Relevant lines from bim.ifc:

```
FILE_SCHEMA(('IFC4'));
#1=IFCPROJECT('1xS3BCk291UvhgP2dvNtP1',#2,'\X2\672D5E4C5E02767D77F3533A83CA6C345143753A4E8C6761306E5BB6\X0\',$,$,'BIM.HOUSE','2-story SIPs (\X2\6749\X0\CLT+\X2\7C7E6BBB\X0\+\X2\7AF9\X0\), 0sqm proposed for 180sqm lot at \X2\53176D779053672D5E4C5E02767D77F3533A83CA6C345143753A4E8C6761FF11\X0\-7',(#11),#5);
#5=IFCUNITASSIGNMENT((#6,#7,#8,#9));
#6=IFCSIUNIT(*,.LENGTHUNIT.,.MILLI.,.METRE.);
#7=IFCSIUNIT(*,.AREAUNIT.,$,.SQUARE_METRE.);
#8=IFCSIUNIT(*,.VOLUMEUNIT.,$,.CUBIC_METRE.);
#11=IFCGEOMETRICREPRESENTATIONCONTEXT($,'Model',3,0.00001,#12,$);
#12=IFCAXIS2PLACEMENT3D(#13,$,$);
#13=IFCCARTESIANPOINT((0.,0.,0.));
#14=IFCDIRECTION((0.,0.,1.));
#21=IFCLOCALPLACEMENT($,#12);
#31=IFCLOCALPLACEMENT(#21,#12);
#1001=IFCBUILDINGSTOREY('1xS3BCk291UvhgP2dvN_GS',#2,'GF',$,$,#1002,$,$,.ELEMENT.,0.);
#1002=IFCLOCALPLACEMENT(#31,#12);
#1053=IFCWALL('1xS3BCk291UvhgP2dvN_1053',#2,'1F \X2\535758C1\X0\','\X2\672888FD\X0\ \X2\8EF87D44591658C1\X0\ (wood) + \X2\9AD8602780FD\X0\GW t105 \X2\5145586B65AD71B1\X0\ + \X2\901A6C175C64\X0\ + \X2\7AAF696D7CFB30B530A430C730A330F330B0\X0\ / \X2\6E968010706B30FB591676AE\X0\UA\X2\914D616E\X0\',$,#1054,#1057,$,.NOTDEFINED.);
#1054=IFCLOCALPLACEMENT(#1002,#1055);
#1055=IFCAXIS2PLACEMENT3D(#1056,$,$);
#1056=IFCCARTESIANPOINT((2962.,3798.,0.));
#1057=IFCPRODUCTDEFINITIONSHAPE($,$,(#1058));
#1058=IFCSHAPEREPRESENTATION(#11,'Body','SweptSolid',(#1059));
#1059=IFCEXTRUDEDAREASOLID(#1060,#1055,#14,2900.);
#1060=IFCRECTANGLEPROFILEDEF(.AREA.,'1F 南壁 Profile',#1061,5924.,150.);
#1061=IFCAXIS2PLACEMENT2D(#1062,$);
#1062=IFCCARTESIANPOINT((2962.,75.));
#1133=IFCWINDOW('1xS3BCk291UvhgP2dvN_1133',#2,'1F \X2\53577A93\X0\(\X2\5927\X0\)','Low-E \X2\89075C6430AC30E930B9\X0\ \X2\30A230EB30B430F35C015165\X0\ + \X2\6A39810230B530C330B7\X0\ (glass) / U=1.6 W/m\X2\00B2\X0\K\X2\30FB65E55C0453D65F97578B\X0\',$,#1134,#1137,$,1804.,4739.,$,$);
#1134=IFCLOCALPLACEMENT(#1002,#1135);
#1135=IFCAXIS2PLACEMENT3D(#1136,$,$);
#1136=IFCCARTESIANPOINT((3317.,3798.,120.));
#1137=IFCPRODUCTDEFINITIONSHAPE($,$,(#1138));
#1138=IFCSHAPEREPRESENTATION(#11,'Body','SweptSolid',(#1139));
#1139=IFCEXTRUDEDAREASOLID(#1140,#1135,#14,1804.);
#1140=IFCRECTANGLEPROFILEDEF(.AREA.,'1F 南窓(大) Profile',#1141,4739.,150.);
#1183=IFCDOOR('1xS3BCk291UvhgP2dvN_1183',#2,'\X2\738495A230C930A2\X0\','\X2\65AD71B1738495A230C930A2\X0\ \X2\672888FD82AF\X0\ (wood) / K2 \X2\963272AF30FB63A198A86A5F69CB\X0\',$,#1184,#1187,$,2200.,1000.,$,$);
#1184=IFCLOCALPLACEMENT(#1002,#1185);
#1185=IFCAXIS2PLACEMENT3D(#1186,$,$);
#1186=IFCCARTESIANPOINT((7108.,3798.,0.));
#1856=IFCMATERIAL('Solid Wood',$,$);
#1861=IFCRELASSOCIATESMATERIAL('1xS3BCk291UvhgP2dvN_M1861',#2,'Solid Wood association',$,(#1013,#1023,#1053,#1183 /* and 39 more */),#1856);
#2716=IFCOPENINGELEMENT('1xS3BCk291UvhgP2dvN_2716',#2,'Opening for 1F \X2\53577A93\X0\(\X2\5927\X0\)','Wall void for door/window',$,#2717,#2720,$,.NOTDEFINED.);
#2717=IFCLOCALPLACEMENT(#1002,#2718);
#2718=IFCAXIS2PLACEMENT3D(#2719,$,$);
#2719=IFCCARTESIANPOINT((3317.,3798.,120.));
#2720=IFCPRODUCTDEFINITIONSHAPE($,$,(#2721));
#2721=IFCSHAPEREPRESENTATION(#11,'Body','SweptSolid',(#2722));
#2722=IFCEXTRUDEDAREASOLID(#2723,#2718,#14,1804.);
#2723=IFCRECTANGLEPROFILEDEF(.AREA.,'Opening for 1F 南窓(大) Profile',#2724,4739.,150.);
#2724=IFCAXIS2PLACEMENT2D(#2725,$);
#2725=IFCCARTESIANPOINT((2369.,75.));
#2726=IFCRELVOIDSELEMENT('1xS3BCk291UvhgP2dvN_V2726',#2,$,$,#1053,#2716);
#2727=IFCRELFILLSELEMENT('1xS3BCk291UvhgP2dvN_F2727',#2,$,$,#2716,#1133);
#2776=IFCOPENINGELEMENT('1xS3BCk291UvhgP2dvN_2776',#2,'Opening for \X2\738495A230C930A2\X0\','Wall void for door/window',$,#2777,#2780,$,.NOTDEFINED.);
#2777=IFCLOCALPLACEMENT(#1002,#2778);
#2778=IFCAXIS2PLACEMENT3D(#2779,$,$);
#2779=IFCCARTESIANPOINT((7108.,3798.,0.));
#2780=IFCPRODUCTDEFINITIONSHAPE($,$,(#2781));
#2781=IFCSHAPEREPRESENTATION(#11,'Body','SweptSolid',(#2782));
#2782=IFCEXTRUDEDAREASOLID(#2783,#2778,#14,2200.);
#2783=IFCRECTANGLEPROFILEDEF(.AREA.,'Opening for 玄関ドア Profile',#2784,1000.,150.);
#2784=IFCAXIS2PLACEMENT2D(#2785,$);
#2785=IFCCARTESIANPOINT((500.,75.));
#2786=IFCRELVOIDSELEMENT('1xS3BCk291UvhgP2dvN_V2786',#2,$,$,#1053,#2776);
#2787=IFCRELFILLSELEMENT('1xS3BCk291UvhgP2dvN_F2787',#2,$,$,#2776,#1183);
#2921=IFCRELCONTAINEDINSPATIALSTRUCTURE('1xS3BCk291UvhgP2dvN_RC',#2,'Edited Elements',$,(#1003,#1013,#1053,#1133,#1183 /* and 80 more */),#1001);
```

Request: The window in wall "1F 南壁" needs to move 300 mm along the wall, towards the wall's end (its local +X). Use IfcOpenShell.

```python
import ifcopenshell
import ifcopenshell.api.geometry
import ifcopenshell.util.placement
import ifcopenshell.util.unit

model = ifcopenshell.open("bim.ifc")
unit_scale = ifcopenshell.util.unit.calculate_unit_scale(model)

window = model.by_guid("1xS3BCk291UvhgP2dvN_1133")
opening = window.FillsVoids[0].RelatingOpeningElement
wall = opening.VoidsElements[0].RelatingBuildingElement

wall_matrix = ifcopenshell.util.placement.get_local_placement(wall.ObjectPlacement)
shift = wall_matrix[:3, 0] * 0.3 / unit_scale
before = ifcopenshell.util.placement.get_local_placement(window.ObjectPlacement)[:3, 3].copy()

# The window is not placed relative to its opening, so move both.
for product in (opening, window):
    matrix = ifcopenshell.util.placement.get_local_placement(product.ObjectPlacement)
    matrix[:3, 3] += shift
    ifcopenshell.api.geometry.edit_object_placement(model, product=product, matrix=matrix, is_si=False)

after = ifcopenshell.util.placement.get_local_placement(window.ObjectPlacement)[:3, 3]
print("window moved by", (after - before).round(3) + 0.0)

model.write("bim_edited.ifc")
```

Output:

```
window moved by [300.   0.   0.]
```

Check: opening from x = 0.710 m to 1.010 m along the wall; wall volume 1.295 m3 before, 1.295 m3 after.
